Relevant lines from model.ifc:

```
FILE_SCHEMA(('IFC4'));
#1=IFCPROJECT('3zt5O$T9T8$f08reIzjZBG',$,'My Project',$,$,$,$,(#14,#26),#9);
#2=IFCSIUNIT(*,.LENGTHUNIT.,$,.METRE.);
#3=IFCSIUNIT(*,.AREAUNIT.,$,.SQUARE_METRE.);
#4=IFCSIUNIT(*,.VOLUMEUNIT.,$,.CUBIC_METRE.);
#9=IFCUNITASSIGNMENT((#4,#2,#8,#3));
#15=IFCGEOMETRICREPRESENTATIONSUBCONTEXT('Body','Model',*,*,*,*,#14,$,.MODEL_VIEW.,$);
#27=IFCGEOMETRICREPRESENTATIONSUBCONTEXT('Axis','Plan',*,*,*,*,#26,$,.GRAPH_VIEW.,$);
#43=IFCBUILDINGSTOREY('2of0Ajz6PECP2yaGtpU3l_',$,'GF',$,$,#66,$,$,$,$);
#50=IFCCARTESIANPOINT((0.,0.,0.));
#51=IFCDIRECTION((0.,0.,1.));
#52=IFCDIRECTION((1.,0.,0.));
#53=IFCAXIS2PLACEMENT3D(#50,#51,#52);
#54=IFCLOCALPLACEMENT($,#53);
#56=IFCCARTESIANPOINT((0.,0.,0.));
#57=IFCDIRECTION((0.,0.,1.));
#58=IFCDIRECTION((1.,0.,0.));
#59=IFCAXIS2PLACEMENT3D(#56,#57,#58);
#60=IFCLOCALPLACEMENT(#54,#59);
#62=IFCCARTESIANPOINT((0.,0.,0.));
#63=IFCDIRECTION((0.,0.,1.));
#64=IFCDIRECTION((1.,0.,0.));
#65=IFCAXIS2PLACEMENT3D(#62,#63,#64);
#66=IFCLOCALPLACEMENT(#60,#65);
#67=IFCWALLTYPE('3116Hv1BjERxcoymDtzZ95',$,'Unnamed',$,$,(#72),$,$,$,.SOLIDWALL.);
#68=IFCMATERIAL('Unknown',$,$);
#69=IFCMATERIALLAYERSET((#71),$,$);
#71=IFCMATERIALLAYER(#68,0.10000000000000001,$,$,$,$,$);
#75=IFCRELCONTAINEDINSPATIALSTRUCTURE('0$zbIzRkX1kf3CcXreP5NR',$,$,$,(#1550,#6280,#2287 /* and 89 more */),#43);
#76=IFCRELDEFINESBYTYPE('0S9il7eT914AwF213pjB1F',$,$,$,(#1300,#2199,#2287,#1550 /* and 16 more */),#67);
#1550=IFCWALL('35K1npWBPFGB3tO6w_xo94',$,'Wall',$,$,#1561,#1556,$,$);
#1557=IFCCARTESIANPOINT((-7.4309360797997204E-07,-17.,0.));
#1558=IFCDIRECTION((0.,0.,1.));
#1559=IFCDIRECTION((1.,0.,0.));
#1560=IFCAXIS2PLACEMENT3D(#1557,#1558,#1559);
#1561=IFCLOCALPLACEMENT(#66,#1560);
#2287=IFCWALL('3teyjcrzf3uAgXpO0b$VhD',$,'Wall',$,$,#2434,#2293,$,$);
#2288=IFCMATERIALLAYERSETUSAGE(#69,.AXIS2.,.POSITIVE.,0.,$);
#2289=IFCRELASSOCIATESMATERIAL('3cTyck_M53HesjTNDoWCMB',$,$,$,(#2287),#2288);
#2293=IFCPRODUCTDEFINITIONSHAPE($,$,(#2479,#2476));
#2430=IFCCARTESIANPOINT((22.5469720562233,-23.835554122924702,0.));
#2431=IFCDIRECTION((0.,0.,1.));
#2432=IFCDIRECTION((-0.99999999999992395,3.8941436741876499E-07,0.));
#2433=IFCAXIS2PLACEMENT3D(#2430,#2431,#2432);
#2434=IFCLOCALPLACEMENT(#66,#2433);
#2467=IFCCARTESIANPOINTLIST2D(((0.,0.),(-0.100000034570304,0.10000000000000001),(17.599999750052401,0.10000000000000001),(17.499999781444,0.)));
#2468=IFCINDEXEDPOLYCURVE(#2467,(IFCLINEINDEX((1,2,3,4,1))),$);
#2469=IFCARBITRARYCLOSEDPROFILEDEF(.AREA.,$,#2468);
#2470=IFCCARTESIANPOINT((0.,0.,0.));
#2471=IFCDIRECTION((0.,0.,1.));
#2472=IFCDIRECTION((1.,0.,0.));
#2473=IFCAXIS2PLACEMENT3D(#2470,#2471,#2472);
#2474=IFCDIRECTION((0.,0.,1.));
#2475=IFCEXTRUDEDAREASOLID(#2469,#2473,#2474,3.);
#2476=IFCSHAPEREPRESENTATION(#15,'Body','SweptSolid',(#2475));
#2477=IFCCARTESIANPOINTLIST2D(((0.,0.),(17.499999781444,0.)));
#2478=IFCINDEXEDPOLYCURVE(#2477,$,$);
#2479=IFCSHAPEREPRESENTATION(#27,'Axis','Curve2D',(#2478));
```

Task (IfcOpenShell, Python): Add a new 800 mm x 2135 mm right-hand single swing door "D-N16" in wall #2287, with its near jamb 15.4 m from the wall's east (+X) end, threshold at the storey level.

```python
import numpy as np
import ifcopenshell
import ifcopenshell.api.feature
import ifcopenshell.api.geometry
import ifcopenshell.api.root
import ifcopenshell.api.spatial
import ifcopenshell.geom
import ifcopenshell.util.element
import ifcopenshell.util.placement
import ifcopenshell.util.representation
import ifcopenshell.util.shape
import ifcopenshell.util.unit

model = ifcopenshell.open("model.ifc")
unit_scale = ifcopenshell.util.unit.calculate_unit_scale(model)
settings = ifcopenshell.geom.settings()


def volume(element):
    """Net volume in cubic metres, openings subtracted."""
    shape = ifcopenshell.geom.create_shape(settings, element)
    return ifcopenshell.util.shape.get_volume(shape.geometry)


wall = model.by_id(2287)
storey = ifcopenshell.util.element.get_container(wall, ifc_class="IfcBuildingStorey")
context = ifcopenshell.util.representation.get_context(model, "Model", "Body", "MODEL_VIEW")
before = volume(wall)

width, height, from_end, sill = 0.8, 2.135, 15.4, 0.0  # metres

# The wall runs along its own X axis, and the end named is its -X end.
wall_shape = ifcopenshell.geom.create_shape(settings, wall)
x, y, z = ifcopenshell.util.shape.get_vertices(wall_shape.geometry).T
start = x.min() + from_end
face, thickness = float(y.min()), float(y.max() - y.min())
wall_matrix = ifcopenshell.util.placement.get_local_placement(wall.ObjectPlacement)
level = ifcopenshell.util.placement.get_local_placement(storey.ObjectPlacement)[2, 3]


def in_wall(x, y):
    """Placement at x, y metres in the wall's axes, at sill height."""
    matrix = wall_matrix.copy()
    matrix[:, 3] = wall_matrix @ np.array([x / unit_scale, y / unit_scale, 0.0, 1.0])
    matrix[2, 3] = level + sill / unit_scale
    return matrix


# Opening: a box that overshoots both wall faces by 50 mm.
opening = ifcopenshell.api.root.create_entity(model, ifc_class="IfcOpeningElement", predefined_type="OPENING")
box = ifcopenshell.api.geometry.add_wall_representation(
    model, context=context, length=width, height=height, thickness=thickness + 0.1
)
ifcopenshell.api.geometry.assign_representation(model, product=opening, representation=box)
ifcopenshell.api.geometry.edit_object_placement(model, product=opening, matrix=in_wall(start, face - 0.05), is_si=False)
ifcopenshell.api.feature.add_feature(model, feature=opening, element=wall)

door = ifcopenshell.api.root.create_entity(model, ifc_class="IfcDoor", name="D-N16", predefined_type="DOOR")
door.OverallWidth, door.OverallHeight = width / unit_scale, height / unit_scale
door.OperationType = "SINGLE_SWING_RIGHT"
body = ifcopenshell.api.geometry.add_door_representation(
    model,
    context=context,
    overall_width=door.OverallWidth,
    overall_height=door.OverallHeight,
    operation_type="SINGLE_SWING_RIGHT",
    lining_properties={"LiningDepth": thickness / unit_scale, "ThresholdDepth": thickness / unit_scale},
)
ifcopenshell.api.geometry.assign_representation(model, product=door, representation=body)
ifcopenshell.api.spatial.assign_container(model, products=[door], relating_structure=storey)
ifcopenshell.api.feature.add_filling(model, opening=opening, element=door)

# The lining spans the wall, so the door starts at the wall face.
ifcopenshell.api.geometry.edit_object_placement(model, product=door, matrix=in_wall(start, face), is_si=False)

after = volume(wall)

print(f"wall volume {before:.3f} -> {after:.3f} m3")

model.write("model-out.ifc")
```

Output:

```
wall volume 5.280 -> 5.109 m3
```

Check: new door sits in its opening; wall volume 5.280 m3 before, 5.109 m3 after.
